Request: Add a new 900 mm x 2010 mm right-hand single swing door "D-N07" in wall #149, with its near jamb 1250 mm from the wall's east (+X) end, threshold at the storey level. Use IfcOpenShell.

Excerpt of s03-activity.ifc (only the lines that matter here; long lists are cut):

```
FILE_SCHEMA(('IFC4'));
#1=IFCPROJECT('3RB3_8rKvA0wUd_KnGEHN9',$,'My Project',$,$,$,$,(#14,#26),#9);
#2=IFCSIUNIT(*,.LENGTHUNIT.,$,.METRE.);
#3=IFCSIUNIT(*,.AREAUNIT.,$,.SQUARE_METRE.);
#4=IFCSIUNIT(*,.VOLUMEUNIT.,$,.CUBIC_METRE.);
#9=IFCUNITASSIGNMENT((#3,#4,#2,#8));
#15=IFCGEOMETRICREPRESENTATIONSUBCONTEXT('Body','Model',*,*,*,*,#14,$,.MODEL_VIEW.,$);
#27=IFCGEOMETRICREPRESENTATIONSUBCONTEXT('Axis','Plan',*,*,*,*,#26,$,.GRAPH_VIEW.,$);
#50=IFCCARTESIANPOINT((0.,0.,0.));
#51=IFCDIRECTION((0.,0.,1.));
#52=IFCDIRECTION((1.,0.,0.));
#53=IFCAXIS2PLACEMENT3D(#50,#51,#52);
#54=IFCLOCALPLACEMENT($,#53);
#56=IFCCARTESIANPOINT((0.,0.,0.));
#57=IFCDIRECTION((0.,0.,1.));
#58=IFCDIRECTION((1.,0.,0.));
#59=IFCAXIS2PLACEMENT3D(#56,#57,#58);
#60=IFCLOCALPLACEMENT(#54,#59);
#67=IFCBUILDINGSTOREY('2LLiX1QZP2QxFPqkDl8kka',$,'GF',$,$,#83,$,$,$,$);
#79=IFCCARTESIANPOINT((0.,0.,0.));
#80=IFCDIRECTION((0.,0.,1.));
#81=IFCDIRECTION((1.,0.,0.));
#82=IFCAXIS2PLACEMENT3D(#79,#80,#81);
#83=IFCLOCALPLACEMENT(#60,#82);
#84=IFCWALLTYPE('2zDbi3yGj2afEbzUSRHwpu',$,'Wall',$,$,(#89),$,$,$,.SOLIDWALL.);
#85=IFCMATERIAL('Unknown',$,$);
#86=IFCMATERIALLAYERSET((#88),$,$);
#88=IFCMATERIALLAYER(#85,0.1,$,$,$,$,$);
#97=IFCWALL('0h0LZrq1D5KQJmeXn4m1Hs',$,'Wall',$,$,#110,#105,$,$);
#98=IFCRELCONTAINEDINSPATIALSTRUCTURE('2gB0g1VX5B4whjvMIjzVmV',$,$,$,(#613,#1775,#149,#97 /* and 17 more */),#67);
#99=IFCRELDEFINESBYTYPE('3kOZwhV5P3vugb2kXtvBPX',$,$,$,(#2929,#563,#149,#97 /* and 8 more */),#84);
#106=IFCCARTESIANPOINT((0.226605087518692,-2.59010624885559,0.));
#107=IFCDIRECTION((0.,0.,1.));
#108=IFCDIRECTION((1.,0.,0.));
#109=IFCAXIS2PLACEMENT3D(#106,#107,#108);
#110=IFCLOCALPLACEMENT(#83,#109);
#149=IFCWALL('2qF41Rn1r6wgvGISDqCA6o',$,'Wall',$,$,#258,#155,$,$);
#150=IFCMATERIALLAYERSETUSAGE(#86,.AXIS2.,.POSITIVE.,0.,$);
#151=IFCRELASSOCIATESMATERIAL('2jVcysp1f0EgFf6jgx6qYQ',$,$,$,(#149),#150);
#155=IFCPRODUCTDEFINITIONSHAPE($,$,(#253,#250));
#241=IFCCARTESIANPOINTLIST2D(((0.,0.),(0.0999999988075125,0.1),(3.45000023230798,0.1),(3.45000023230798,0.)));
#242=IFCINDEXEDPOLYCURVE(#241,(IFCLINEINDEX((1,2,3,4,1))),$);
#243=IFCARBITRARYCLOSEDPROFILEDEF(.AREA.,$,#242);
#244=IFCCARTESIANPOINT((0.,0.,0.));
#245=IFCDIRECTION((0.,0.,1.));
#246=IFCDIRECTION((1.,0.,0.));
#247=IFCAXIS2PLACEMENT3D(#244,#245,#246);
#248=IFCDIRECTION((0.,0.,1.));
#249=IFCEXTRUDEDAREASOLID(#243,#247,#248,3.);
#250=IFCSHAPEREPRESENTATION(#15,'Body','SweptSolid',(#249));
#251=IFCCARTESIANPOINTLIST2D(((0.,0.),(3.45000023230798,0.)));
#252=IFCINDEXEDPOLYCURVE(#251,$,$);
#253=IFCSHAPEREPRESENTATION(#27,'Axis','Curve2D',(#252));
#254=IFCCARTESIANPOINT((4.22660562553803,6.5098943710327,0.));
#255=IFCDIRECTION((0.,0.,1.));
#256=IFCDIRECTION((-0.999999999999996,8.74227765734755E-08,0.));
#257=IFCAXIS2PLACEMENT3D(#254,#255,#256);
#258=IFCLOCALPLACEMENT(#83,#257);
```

```python
import numpy as np
import ifcopenshell
import ifcopenshell.api.feature
import ifcopenshell.api.geometry
import ifcopenshell.api.root
import ifcopenshell.api.spatial
import ifcopenshell.geom
import ifcopenshell.util.element
import ifcopenshell.util.placement
import ifcopenshell.util.representation
import ifcopenshell.util.shape
import ifcopenshell.util.unit

model = ifcopenshell.open("s03-activity.ifc")
unit_scale = ifcopenshell.util.unit.calculate_unit_scale(model)
settings = ifcopenshell.geom.settings()


def volume(element):
    """Net volume in cubic metres, openings subtracted."""
    shape = ifcopenshell.geom.create_shape(settings, element)
    return ifcopenshell.util.shape.get_volume(shape.geometry)


wall = model.by_guid("2qF41Rn1r6wgvGISDqCA6o")
storey = ifcopenshell.util.element.get_container(wall, ifc_class="IfcBuildingStorey")
context = ifcopenshell.util.representation.get_context(model, "Model", "Body", "MODEL_VIEW")
before = volume(wall)

width, height, from_end, sill = 0.9, 2.01, 1.25, 0.0  # metres

# The wall runs along its own X axis, and the end named is its -X end.
wall_shape = ifcopenshell.geom.create_shape(settings, wall)
x, y, z = ifcopenshell.util.shape.get_vertices(wall_shape.geometry).T
start = x.min() + from_end
face, thickness = float(y.min()), float(y.max() - y.min())
wall_matrix = ifcopenshell.util.placement.get_local_placement(wall.ObjectPlacement)
level = ifcopenshell.util.placement.get_local_placement(storey.ObjectPlacement)[2, 3]


def in_wall(x, y):
    """Placement at x, y metres in the wall's axes, at sill height."""
    matrix = wall_matrix.copy()
    matrix[:, 3] = wall_matrix @ np.array([x / unit_scale, y / unit_scale, 0.0, 1.0])
    matrix[2, 3] = level + sill / unit_scale
    return matrix


# Opening: a box that overshoots both wall faces by 50 mm.
opening = ifcopenshell.api.root.create_entity(model, ifc_class="IfcOpeningElement", predefined_type="OPENING")
box = ifcopenshell.api.geometry.add_wall_representation(
    model, context=context, length=width, height=height, thickness=thickness + 0.1
)
ifcopenshell.api.geometry.assign_representation(model, product=opening, representation=box)
ifcopenshell.api.geometry.edit_object_placement(model, product=opening, matrix=in_wall(start, face - 0.05), is_si=False)
ifcopenshell.api.feature.add_feature(model, feature=opening, element=wall)

door = ifcopenshell.api.root.create_entity(model, ifc_class="IfcDoor", name="D-N07", predefined_type="DOOR")
door.OverallWidth, door.OverallHeight = width / unit_scale, height / unit_scale
door.OperationType = "SINGLE_SWING_RIGHT"
body = ifcopenshell.api.geometry.add_door_representation(
    model,
    context=context,
    overall_width=door.OverallWidth,
    overall_height=door.OverallHeight,
    operation_type="SINGLE_SWING_RIGHT",
    lining_properties={"LiningDepth": thickness / unit_scale, "ThresholdDepth": thickness / unit_scale},
)
ifcopenshell.api.geometry.assign_representation(model, product=door, representation=body)
ifcopenshell.api.spatial.assign_container(model, products=[door], relating_structure=storey)
ifcopenshell.api.feature.add_filling(model, opening=opening, element=door)

# The lining spans the wall, so the door starts at the wall face.
ifcopenshell.api.geometry.edit_object_placement(model, product=door, matrix=in_wall(start, face), is_si=False)

after = volume(wall)

print(f"wall volume {before:.3f} -> {after:.3f} m3")

model.write("s03-activity_edited.ifc")
```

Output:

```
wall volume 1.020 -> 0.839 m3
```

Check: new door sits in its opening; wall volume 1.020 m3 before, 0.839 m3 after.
